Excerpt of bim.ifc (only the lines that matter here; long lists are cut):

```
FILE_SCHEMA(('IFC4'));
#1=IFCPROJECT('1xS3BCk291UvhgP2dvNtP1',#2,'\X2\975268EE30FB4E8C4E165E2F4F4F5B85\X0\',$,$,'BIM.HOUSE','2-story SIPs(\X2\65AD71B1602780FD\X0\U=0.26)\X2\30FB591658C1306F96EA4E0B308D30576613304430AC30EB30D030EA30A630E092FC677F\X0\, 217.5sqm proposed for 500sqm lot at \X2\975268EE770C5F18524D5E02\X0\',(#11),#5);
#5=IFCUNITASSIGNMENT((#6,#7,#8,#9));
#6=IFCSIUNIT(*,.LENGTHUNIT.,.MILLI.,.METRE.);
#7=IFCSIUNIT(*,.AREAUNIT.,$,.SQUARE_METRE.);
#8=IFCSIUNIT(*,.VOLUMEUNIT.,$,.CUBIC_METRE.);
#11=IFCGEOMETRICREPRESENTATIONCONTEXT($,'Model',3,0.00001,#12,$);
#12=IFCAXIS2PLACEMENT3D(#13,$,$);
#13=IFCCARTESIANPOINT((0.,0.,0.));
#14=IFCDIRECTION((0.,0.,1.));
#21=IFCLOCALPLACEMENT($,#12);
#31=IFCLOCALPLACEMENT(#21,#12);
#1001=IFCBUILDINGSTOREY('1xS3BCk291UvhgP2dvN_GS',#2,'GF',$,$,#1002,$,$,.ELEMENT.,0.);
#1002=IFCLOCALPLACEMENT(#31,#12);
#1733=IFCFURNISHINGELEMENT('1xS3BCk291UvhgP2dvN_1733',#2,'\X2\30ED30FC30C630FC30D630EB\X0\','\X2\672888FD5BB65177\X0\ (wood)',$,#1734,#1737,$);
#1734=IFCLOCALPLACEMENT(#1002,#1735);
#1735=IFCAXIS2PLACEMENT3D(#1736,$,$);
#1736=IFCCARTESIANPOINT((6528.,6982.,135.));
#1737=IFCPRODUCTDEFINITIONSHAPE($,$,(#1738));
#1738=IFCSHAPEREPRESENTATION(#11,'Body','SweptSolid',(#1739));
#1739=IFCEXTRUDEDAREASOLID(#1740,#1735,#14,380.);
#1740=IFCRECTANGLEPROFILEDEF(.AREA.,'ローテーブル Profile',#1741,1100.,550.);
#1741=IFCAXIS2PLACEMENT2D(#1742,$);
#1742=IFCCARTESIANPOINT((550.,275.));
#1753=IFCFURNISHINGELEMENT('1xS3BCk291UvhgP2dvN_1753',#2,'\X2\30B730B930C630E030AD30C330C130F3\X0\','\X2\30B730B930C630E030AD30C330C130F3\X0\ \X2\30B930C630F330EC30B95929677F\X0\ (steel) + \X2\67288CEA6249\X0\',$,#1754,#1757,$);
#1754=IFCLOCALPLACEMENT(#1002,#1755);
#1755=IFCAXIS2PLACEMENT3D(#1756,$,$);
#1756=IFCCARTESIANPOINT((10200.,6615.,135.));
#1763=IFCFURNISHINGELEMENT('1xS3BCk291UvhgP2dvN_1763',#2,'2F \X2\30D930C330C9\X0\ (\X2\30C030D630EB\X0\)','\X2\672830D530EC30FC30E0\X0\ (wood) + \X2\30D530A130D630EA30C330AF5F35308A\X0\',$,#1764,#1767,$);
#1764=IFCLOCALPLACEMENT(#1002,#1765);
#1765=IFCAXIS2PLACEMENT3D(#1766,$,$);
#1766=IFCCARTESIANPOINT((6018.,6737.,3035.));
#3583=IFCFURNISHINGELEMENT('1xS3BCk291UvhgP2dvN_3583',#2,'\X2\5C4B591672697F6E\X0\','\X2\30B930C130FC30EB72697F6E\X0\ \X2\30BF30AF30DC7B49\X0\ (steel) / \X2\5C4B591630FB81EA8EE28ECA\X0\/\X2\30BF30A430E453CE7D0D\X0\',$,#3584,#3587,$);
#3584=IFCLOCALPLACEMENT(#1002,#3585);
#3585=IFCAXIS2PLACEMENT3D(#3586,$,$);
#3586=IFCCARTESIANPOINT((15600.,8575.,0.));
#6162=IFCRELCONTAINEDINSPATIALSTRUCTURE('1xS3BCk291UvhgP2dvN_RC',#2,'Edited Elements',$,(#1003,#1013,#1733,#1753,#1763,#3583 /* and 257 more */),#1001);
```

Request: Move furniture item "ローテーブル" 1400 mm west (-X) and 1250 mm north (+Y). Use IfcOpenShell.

```python
import ifcopenshell
import ifcopenshell.api.geometry
import ifcopenshell.util.placement

model = ifcopenshell.open("bim.ifc")

item = model.by_guid("1xS3BCk291UvhgP2dvN_1733")
matrix = ifcopenshell.util.placement.get_local_placement(item.ObjectPlacement)
matrix[0, 3] -= 1400.0
matrix[1, 3] += 1250.0
ifcopenshell.api.geometry.edit_object_placement(model, product=item, matrix=matrix, is_si=False)

print(ifcopenshell.util.placement.get_local_placement(item.ObjectPlacement).round(3) + 0.0)

model.write("bim_updated.ifc")
```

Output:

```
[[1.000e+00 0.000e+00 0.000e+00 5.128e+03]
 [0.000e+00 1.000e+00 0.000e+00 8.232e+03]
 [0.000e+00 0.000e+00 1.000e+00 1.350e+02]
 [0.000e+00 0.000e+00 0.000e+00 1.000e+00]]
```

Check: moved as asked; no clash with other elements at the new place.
